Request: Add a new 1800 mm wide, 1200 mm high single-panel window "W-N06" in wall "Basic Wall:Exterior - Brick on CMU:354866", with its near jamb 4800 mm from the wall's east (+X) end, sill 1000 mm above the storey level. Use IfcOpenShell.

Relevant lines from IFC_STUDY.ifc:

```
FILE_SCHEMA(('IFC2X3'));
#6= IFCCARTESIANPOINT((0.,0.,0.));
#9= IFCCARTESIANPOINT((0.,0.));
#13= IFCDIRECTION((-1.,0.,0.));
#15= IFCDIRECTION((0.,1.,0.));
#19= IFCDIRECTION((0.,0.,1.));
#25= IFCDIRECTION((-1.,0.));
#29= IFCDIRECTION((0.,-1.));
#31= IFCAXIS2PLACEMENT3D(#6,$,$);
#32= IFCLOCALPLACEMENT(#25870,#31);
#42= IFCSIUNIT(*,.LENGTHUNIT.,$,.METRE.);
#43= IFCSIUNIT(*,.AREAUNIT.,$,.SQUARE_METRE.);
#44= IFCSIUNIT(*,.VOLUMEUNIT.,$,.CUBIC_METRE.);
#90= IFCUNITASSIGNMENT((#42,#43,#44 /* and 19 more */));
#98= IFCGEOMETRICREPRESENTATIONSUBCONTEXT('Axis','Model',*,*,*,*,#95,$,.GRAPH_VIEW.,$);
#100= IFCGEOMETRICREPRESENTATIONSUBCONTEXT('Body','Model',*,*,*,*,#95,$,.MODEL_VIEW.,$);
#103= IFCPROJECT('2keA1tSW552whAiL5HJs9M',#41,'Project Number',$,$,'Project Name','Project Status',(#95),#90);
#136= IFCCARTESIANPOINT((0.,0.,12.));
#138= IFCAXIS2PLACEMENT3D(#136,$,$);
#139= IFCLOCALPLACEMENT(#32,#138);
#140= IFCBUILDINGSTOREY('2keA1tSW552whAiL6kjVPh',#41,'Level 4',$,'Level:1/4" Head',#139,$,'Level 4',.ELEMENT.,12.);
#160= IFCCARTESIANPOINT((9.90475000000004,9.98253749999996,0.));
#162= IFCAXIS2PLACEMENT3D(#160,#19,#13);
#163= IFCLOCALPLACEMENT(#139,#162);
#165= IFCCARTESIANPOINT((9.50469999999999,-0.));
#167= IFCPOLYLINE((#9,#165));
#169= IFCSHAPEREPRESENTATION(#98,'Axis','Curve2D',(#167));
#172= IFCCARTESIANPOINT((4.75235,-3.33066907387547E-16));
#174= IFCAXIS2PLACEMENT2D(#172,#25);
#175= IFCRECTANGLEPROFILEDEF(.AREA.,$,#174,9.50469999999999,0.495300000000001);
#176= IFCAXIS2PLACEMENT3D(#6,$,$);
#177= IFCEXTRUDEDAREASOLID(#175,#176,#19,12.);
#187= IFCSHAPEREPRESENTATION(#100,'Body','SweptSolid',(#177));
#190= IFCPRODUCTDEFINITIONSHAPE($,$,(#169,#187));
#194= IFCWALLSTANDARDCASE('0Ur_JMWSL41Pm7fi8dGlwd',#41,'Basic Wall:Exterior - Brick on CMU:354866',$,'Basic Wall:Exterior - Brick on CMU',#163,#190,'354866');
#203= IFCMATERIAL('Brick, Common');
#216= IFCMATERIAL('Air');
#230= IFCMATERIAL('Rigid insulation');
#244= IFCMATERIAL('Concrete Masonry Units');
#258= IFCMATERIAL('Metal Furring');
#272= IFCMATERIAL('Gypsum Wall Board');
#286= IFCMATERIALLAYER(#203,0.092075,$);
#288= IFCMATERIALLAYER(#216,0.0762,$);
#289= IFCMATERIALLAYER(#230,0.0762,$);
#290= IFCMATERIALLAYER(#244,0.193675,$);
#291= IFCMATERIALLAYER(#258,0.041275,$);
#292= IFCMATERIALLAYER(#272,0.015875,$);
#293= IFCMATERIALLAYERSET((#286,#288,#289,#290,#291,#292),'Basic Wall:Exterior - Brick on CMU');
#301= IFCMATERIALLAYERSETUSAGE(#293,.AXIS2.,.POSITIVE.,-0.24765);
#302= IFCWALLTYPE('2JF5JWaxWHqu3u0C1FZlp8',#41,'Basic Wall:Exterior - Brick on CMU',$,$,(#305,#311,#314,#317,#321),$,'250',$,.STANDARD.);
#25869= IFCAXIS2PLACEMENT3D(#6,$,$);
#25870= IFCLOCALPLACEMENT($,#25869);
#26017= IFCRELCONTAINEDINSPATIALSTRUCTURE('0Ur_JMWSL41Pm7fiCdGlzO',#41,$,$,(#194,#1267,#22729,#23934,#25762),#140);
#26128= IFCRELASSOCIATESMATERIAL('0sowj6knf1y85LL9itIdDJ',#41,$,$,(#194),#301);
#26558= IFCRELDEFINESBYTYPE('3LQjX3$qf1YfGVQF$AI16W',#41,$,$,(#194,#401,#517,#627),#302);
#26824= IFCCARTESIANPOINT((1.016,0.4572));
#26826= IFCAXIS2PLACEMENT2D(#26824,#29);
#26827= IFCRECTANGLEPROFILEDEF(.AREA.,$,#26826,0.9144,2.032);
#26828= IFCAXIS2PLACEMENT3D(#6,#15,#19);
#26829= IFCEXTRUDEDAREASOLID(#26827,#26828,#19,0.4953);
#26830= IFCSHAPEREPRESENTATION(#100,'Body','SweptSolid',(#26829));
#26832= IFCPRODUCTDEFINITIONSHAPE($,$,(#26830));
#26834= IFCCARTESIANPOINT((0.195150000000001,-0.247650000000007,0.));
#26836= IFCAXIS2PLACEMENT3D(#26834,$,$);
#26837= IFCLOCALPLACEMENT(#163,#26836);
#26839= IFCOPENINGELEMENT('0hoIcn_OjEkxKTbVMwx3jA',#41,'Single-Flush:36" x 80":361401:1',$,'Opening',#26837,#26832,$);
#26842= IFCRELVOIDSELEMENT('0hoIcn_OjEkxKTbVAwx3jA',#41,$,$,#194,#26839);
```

```python
import numpy as np
import ifcopenshell
import ifcopenshell.api.feature
import ifcopenshell.api.geometry
import ifcopenshell.api.root
import ifcopenshell.api.spatial
import ifcopenshell.api.type
import ifcopenshell.geom
import ifcopenshell.util.element
import ifcopenshell.util.placement
import ifcopenshell.util.representation
import ifcopenshell.util.shape
import ifcopenshell.util.unit

model = ifcopenshell.open("IFC_STUDY.ifc")
unit_scale = ifcopenshell.util.unit.calculate_unit_scale(model)
settings = ifcopenshell.geom.settings()


def volume(element):
    """Net volume in cubic metres, openings subtracted."""
    shape = ifcopenshell.geom.create_shape(settings, element)
    return ifcopenshell.util.shape.get_volume(shape.geometry)


wall = model.by_guid("0Ur_JMWSL41Pm7fi8dGlwd")
storey = ifcopenshell.util.element.get_container(wall, ifc_class="IfcBuildingStorey")
context = ifcopenshell.util.representation.get_context(model, "Model", "Body", "MODEL_VIEW")
before = volume(wall)

width, height, from_end, sill = 1.8, 1.2, 4.8, 1  # metres

# The wall runs along its own X axis, and the end named is its -X end.
wall_shape = ifcopenshell.geom.create_shape(settings, wall)
x, y, z = ifcopenshell.util.shape.get_vertices(wall_shape.geometry).T
start = x.min() + from_end
face, thickness = float(y.min()), float(y.max() - y.min())
wall_matrix = ifcopenshell.util.placement.get_local_placement(wall.ObjectPlacement)
level = ifcopenshell.util.placement.get_local_placement(storey.ObjectPlacement)[2, 3]


def in_wall(x, y):
    """Placement at x, y metres in the wall's axes, at sill height."""
    matrix = wall_matrix.copy()
    matrix[:, 3] = wall_matrix @ np.array([x / unit_scale, y / unit_scale, 0.0, 1.0])
    matrix[2, 3] = level + sill / unit_scale
    return matrix


# Opening: a box that overshoots both wall faces by 50 mm.
opening = ifcopenshell.api.root.create_entity(model, ifc_class="IfcOpeningElement")
box = ifcopenshell.api.geometry.add_wall_representation(
    model, context=context, length=width, height=height, thickness=thickness + 0.1
)
ifcopenshell.api.geometry.assign_representation(model, product=opening, representation=box)
ifcopenshell.api.geometry.edit_object_placement(model, product=opening, matrix=in_wall(start, face - 0.05), is_si=False)
ifcopenshell.api.feature.add_feature(model, feature=opening, element=wall)

window = ifcopenshell.api.root.create_entity(model, ifc_class="IfcWindow", name="W-N06")
window.OverallWidth, window.OverallHeight = width / unit_scale, height / unit_scale
body = ifcopenshell.api.geometry.add_window_representation(
    model,
    context=context,
    overall_width=window.OverallWidth,
    overall_height=window.OverallHeight,
    partition_type="SINGLE_PANEL",
)
ifcopenshell.api.geometry.assign_representation(model, product=window, representation=body)
ifcopenshell.api.spatial.assign_container(model, products=[window], relating_structure=storey)
fills = ifcopenshell.api.feature.add_filling(model, opening=opening, element=window)
fills.OwnerHistory = window.OwnerHistory  # required in IFC2X3

# IFC2X3 keeps the operation on the window style.
style = ifcopenshell.api.root.create_entity(model, ifc_class="IfcWindowStyle", name="W-N06")
style.OperationType, style.ConstructionType = "SINGLE_PANEL", "NOTDEFINED"
style.ParameterTakesPrecedence = style.Sizeable = False
ifcopenshell.api.type.assign_type(model, related_objects=[window], relating_type=style)

# Centre the window in the wall's thickness.
ifcopenshell.api.geometry.edit_object_placement(model, product=window, matrix=in_wall(start, face), is_si=False)
window_shape = ifcopenshell.geom.create_shape(settings, window)
depth = ifcopenshell.util.shape.get_vertices(window_shape.geometry)[:, 1]
offset = face + thickness / 2 - (depth.min() + depth.max()) / 2
ifcopenshell.api.geometry.edit_object_placement(model, product=window, matrix=in_wall(start, offset), is_si=False)

after = volume(wall)

print(f"wall volume {before:.3f} -> {after:.3f} m3")

model.write("IFC_STUDY_updated.ifc")
```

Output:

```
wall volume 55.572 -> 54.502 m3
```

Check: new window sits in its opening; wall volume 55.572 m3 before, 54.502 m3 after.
